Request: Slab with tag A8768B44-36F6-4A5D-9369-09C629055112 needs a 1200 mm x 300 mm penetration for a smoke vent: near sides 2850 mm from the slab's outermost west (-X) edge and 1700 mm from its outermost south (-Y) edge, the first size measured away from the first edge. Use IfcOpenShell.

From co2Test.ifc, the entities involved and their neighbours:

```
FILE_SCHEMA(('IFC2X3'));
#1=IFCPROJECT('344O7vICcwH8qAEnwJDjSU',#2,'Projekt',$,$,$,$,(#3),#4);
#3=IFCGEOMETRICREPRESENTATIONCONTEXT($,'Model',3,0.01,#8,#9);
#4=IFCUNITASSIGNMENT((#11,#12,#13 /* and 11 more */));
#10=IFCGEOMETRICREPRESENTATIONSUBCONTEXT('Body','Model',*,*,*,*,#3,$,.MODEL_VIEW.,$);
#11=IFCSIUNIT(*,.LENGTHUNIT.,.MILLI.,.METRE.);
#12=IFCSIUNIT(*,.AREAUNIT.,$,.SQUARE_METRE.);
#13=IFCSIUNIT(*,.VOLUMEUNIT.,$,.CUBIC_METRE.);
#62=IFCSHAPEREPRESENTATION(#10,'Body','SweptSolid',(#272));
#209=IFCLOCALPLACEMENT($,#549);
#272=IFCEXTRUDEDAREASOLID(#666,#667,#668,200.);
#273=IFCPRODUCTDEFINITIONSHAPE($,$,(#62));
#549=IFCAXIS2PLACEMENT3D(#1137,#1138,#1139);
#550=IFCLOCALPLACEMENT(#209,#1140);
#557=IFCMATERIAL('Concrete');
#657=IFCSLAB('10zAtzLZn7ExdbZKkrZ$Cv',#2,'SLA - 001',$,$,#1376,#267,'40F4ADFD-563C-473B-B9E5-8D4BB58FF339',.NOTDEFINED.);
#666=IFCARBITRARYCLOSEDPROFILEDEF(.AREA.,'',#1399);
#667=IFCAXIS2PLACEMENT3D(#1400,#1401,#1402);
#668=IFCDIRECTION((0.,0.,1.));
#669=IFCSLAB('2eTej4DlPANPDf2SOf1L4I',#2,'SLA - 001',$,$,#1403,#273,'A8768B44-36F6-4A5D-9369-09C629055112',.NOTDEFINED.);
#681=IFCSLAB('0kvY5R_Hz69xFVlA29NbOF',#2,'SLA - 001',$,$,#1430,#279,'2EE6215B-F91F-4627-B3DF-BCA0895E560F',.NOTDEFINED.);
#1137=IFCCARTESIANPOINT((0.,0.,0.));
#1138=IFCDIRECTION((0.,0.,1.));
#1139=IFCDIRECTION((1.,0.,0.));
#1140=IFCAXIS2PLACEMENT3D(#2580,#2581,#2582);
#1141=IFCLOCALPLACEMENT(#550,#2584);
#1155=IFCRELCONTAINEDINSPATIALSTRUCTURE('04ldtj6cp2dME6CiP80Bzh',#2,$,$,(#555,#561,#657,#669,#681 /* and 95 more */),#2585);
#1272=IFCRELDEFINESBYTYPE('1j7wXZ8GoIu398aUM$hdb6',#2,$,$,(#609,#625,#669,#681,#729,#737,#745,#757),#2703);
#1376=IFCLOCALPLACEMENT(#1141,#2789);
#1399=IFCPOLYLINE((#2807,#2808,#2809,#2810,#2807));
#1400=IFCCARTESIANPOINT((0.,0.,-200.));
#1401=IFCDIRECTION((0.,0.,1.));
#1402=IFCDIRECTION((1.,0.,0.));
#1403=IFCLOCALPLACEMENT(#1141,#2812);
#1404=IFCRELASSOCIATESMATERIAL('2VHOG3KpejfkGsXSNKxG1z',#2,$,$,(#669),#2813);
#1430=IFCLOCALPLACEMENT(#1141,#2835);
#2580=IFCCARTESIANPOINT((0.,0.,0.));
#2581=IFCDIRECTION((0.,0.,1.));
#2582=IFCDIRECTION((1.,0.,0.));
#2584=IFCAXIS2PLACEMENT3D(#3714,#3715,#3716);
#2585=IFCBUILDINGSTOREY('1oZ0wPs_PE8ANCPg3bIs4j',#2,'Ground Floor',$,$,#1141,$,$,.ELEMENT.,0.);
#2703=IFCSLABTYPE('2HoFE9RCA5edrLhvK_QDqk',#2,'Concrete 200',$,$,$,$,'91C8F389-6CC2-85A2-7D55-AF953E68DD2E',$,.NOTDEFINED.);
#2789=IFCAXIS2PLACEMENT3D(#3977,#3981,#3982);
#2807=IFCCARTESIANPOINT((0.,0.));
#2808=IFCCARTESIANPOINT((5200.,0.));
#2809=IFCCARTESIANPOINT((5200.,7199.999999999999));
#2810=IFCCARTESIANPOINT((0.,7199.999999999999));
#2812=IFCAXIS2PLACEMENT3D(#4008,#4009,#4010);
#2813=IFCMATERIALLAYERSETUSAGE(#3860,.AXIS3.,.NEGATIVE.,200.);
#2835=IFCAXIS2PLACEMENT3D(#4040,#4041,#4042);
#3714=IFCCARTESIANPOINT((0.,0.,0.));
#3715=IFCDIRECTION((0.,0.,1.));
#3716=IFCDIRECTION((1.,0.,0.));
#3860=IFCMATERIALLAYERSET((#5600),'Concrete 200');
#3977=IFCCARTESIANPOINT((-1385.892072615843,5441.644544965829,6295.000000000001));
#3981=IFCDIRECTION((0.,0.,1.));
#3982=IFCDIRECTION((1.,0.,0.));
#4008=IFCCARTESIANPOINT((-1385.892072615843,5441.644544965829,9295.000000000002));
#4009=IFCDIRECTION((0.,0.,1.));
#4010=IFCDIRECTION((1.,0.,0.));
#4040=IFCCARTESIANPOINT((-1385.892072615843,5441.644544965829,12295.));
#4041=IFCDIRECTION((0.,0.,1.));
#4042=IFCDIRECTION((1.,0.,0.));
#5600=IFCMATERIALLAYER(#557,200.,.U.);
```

```python
import numpy as np
import ifcopenshell
import ifcopenshell.api.feature
import ifcopenshell.api.geometry
import ifcopenshell.api.root
import ifcopenshell.geom
import ifcopenshell.util.placement
import ifcopenshell.util.representation
import ifcopenshell.util.shape
import ifcopenshell.util.unit

model = ifcopenshell.open("co2Test.ifc")
unit_scale = ifcopenshell.util.unit.calculate_unit_scale(model)
settings = ifcopenshell.geom.settings()


def volume(element):
    """Net volume in cubic metres, openings subtracted."""
    shape = ifcopenshell.geom.create_shape(settings, element)
    return ifcopenshell.util.shape.get_volume(shape.geometry)


slab = model.by_guid("2eTej4DlPANPDf2SOf1L4I")
before = volume(slab)

# Extent in the slab's own axes, in metres. The edges named are its -X and -Y sides.
slab_shape = ifcopenshell.geom.create_shape(settings, slab)
vertices = ifcopenshell.util.shape.get_vertices(slab_shape.geometry)
x_min, y_min, bottom = vertices.min(axis=0)
top = vertices[:, 2].max()

opening = ifcopenshell.api.root.create_entity(model, ifc_class="IfcOpeningElement", name="Smoke vent opening")
context = ifcopenshell.util.representation.get_context(model, "Model", "Body", "MODEL_VIEW")
width, depth = 1.2, 0.3
outline = [(0.0, 0.0), (width, 0.0), (width, depth), (0.0, depth), (0.0, 0.0)]
# Overshoot both faces by 50 mm so the cut is clean.
shape = ifcopenshell.api.geometry.add_slab_representation(
    model, context=context, depth=top - bottom + 0.1, polyline=outline
)
ifcopenshell.api.geometry.assign_representation(model, product=opening, representation=shape)

matrix = ifcopenshell.util.placement.get_local_placement(slab.ObjectPlacement)
matrix[:, 3] = matrix @ np.append(np.array([x_min + 2.85, y_min + 1.7, bottom - 0.05]) / unit_scale, 1.0)
ifcopenshell.api.geometry.edit_object_placement(model, product=opening, matrix=matrix, is_si=False)
ifcopenshell.api.feature.add_feature(model, feature=opening, element=slab)

after = volume(slab)

print(f"slab volume {before:.3f} -> {after:.3f} m3")

model.write("co2Test-out.ifc")
```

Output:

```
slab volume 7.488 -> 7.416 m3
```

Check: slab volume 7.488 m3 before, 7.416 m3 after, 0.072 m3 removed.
